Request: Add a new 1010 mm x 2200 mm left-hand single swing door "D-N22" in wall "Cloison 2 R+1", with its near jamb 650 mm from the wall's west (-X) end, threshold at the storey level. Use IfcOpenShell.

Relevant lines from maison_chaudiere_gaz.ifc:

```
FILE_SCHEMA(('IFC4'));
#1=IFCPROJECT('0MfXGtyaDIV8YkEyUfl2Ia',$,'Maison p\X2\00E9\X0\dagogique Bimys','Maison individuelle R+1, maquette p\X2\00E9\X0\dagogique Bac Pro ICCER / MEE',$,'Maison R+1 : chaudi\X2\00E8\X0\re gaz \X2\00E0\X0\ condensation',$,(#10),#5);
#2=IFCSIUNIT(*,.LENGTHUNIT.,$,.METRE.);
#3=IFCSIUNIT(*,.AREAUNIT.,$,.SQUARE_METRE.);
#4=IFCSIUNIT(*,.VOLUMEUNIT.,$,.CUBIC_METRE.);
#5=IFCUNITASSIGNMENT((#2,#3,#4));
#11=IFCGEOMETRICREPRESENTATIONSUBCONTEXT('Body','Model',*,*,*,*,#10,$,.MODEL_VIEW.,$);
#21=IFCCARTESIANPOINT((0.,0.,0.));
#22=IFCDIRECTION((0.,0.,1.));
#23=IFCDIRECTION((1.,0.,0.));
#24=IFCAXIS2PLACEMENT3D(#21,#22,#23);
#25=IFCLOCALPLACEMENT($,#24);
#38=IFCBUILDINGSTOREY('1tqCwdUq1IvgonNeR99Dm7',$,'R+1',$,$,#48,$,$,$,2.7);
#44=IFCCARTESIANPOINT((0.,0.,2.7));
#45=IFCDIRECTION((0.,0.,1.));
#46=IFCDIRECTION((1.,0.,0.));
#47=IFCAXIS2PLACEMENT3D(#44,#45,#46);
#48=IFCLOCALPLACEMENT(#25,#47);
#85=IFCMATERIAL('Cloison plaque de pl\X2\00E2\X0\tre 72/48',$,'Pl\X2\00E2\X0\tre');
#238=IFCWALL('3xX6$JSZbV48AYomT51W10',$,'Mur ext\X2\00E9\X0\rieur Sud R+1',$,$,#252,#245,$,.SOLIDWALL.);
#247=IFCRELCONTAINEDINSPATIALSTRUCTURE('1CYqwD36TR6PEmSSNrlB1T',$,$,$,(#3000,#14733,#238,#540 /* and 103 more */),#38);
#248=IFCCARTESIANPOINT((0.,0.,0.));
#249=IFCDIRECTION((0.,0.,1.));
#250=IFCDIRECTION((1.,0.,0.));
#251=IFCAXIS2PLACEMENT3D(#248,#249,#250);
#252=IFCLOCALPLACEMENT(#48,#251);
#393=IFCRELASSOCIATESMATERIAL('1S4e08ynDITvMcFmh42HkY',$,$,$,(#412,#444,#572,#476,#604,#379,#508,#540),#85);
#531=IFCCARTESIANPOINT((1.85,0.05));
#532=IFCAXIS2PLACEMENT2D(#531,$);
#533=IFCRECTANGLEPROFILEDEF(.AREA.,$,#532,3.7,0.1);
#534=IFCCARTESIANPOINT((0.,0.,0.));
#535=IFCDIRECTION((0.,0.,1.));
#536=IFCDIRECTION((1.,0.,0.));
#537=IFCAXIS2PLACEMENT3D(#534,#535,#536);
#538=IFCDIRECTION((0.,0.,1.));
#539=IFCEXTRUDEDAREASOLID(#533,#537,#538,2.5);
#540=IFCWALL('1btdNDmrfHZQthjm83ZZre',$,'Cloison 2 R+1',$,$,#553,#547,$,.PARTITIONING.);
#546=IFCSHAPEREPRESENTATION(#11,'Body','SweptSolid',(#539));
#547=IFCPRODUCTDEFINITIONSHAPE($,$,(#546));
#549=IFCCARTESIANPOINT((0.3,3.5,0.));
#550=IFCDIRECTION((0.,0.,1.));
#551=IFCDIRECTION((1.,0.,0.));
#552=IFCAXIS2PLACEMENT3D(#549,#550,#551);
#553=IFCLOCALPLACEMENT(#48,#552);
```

```python
import numpy as np
import ifcopenshell
import ifcopenshell.api.feature
import ifcopenshell.api.geometry
import ifcopenshell.api.root
import ifcopenshell.api.spatial
import ifcopenshell.geom
import ifcopenshell.util.element
import ifcopenshell.util.placement
import ifcopenshell.util.representation
import ifcopenshell.util.shape
import ifcopenshell.util.unit

model = ifcopenshell.open("maison_chaudiere_gaz.ifc")
unit_scale = ifcopenshell.util.unit.calculate_unit_scale(model)
settings = ifcopenshell.geom.settings()


def volume(element):
    """Net volume in cubic metres, openings subtracted."""
    shape = ifcopenshell.geom.create_shape(settings, element)
    return ifcopenshell.util.shape.get_volume(shape.geometry)


wall = model.by_guid("1btdNDmrfHZQthjm83ZZre")
storey = ifcopenshell.util.element.get_container(wall, ifc_class="IfcBuildingStorey")
context = ifcopenshell.util.representation.get_context(model, "Model", "Body", "MODEL_VIEW")
before = volume(wall)

width, height, from_end, sill = 1.01, 2.2, 0.65, 0.0  # metres

# The wall runs along its own X axis, and the end named is its -X end.
wall_shape = ifcopenshell.geom.create_shape(settings, wall)
x, y, z = ifcopenshell.util.shape.get_vertices(wall_shape.geometry).T
start = x.min() + from_end
face, thickness = float(y.min()), float(y.max() - y.min())
wall_matrix = ifcopenshell.util.placement.get_local_placement(wall.ObjectPlacement)
level = ifcopenshell.util.placement.get_local_placement(storey.ObjectPlacement)[2, 3]


def in_wall(x, y):
    """Placement at x, y metres in the wall's axes, at sill height."""
    matrix = wall_matrix.copy()
    matrix[:, 3] = wall_matrix @ np.array([x / unit_scale, y / unit_scale, 0.0, 1.0])
    matrix[2, 3] = level + sill / unit_scale
    return matrix


# Opening: a box that overshoots both wall faces by 50 mm.
opening = ifcopenshell.api.root.create_entity(model, ifc_class="IfcOpeningElement", predefined_type="OPENING")
box = ifcopenshell.api.geometry.add_wall_representation(
    model, context=context, length=width, height=height, thickness=thickness + 0.1
)
ifcopenshell.api.geometry.assign_representation(model, product=opening, representation=box)
ifcopenshell.api.geometry.edit_object_placement(model, product=opening, matrix=in_wall(start, face - 0.05), is_si=False)
ifcopenshell.api.feature.add_feature(model, feature=opening, element=wall)

door = ifcopenshell.api.root.create_entity(model, ifc_class="IfcDoor", name="D-N22", predefined_type="DOOR")
door.OverallWidth, door.OverallHeight = width / unit_scale, height / unit_scale
door.OperationType = "SINGLE_SWING_LEFT"
body = ifcopenshell.api.geometry.add_door_representation(
    model,
    context=context,
    overall_width=door.OverallWidth,
    overall_height=door.OverallHeight,
    operation_type="SINGLE_SWING_LEFT",
    lining_properties={"LiningDepth": thickness / unit_scale, "ThresholdDepth": thickness / unit_scale},
)
ifcopenshell.api.geometry.assign_representation(model, product=door, representation=body)
ifcopenshell.api.spatial.assign_container(model, products=[door], relating_structure=storey)
ifcopenshell.api.feature.add_filling(model, opening=opening, element=door)

# The lining spans the wall, so the door starts at the wall face.
ifcopenshell.api.geometry.edit_object_placement(model, product=door, matrix=in_wall(start, face), is_si=False)

after = volume(wall)

print(f"wall volume {before:.3f} -> {after:.3f} m3")

model.write("maison_chaudiere_gaz_updated.ifc")
```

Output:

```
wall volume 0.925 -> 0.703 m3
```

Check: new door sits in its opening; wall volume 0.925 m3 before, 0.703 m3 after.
